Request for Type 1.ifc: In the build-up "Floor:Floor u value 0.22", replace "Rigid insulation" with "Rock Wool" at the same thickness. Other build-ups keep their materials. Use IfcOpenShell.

First a look at what the model holds.

```python
import ifcopenshell
import ifcopenshell.util.element

model = ifcopenshell.open("Type 1.ifc")
print(model.schema)
for layer_set in model.by_type("IfcMaterialLayerSet"):
    if layer_set.LayerSetName == "Floor:Floor u value 0.22":
        for layer in layer_set.MaterialLayers:
            print(layer.id(), layer.Material and layer.Material.Name, layer.LayerThickness, sep=" | ")
        print(len(ifcopenshell.util.element.get_elements_by_material(model, layer_set)), "elements and types use it")
print(sorted(m.Name for m in model.by_type("IfcMaterial") if m.Name)[:60])
```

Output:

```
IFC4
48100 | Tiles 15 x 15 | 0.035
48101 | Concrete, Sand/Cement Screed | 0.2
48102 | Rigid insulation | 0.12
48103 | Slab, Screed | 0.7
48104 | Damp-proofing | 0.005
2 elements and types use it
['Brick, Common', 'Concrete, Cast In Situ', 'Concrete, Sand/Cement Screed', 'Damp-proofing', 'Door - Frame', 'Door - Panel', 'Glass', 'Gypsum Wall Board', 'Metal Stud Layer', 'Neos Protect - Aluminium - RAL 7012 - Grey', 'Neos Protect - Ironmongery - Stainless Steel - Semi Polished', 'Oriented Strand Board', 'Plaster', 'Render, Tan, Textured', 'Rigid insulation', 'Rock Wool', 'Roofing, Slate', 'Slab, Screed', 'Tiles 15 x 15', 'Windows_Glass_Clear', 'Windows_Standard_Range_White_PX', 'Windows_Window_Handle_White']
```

```python
import ifcopenshell
import ifcopenshell.api.material

model = ifcopenshell.open("Type 1.ifc")

layer_set = next(s for s in model.by_type("IfcMaterialLayerSet") if s.LayerSetName == "Floor:Floor u value 0.22")
layer = next(l for l in layer_set.MaterialLayers if l.Material and l.Material.Name == "Rigid insulation")
material = next(m for m in model.by_type("IfcMaterial") if m.Name == "Rock Wool")

# Point this one layer at the other material; renaming the old one would change it everywhere.
ifcopenshell.api.material.edit_layer(model, layer=layer, attributes={"Name": material.Name}, material=material)

print([l.Material.Name if l.Material else None for l in layer_set.MaterialLayers])

model.write("Type 1_rev.ifc")
```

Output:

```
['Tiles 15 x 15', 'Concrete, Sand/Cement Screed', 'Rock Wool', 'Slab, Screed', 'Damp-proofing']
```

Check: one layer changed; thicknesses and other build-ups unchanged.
